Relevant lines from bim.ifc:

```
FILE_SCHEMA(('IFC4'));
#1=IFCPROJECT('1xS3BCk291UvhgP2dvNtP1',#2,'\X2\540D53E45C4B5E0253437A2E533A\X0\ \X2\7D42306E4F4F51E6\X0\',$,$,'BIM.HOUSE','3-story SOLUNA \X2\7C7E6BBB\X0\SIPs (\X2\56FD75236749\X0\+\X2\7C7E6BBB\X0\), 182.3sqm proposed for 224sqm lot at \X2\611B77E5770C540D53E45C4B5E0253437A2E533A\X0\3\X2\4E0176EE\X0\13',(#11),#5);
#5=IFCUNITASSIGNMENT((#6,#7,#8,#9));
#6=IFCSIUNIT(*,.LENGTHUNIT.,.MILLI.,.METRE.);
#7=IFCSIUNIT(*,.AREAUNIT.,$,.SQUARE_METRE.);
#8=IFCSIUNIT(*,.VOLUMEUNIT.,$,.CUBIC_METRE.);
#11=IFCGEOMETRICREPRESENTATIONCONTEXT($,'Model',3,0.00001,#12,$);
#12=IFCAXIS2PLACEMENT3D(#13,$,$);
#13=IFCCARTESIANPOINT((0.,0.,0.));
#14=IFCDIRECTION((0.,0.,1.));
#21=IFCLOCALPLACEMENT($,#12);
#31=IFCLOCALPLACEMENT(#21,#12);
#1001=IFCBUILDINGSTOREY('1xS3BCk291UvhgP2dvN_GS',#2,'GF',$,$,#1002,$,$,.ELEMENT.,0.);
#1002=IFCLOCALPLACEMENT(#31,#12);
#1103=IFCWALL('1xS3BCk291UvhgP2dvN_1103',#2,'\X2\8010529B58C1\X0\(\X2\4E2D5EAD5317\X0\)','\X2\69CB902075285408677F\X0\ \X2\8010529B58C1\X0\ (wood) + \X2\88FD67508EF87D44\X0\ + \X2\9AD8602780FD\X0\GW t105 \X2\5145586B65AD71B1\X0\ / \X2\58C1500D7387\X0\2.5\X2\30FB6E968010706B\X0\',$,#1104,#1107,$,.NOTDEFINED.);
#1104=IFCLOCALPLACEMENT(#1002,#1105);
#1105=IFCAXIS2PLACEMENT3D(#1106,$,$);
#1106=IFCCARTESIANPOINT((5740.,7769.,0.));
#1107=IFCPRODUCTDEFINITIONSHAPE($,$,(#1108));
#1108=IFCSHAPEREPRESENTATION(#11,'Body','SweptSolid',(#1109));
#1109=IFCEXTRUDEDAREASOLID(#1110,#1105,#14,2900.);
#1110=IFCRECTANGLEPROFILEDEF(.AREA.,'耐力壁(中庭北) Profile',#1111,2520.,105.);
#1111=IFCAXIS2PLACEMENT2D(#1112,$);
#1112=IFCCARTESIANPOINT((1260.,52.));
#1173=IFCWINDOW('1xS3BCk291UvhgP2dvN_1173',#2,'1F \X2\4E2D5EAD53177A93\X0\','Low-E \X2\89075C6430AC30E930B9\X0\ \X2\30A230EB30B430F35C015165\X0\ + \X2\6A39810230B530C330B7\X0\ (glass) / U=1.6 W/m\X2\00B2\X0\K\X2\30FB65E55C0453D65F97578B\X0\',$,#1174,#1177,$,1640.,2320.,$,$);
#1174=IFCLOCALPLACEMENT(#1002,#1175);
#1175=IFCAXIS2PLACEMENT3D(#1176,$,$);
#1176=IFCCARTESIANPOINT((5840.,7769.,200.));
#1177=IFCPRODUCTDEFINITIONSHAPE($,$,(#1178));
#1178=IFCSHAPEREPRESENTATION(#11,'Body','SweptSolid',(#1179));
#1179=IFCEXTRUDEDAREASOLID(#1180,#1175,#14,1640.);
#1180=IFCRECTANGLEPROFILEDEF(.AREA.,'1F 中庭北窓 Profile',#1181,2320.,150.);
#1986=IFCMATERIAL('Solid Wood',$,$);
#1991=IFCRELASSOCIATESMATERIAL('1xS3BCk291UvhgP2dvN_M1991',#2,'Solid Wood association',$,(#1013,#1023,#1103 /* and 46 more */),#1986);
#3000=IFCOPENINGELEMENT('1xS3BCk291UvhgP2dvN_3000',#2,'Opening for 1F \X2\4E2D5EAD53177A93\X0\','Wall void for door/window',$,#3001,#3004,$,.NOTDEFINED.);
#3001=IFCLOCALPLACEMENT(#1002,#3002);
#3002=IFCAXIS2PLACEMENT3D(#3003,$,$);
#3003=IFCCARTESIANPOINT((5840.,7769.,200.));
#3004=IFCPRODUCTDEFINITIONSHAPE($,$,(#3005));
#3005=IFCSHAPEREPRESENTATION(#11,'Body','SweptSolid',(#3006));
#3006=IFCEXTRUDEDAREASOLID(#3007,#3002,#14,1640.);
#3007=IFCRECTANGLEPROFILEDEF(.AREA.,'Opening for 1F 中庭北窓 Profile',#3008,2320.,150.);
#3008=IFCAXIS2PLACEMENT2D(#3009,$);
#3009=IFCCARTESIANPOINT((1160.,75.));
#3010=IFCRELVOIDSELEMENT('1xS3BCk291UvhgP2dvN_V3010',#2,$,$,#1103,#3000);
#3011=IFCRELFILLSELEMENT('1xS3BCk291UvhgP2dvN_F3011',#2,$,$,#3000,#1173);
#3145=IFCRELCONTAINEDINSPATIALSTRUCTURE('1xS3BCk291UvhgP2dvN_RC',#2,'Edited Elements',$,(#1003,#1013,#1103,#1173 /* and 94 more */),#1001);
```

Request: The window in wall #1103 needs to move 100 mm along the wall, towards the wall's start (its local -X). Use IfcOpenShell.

```python
import ifcopenshell
import ifcopenshell.api.geometry
import ifcopenshell.util.placement

model = ifcopenshell.open("bim.ifc")

window = model.by_id(1173)
opening = window.FillsVoids[0].RelatingOpeningElement
wall = opening.VoidsElements[0].RelatingBuildingElement

wall_matrix = ifcopenshell.util.placement.get_local_placement(wall.ObjectPlacement)
shift = wall_matrix[:3, 0] * -100.0
before = ifcopenshell.util.placement.get_local_placement(window.ObjectPlacement)[:3, 3].copy()

# The window is not placed relative to its opening, so move both.
for product in (opening, window):
    matrix = ifcopenshell.util.placement.get_local_placement(product.ObjectPlacement)
    matrix[:3, 3] += shift
    ifcopenshell.api.geometry.edit_object_placement(model, product=product, matrix=matrix, is_si=False)

after = ifcopenshell.util.placement.get_local_placement(window.ObjectPlacement)[:3, 3]
print("window moved by", (after - before).round(3) + 0.0)

model.write("bim-out.ifc")
```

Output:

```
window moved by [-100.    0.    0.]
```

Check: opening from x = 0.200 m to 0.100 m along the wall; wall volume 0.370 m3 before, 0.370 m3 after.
